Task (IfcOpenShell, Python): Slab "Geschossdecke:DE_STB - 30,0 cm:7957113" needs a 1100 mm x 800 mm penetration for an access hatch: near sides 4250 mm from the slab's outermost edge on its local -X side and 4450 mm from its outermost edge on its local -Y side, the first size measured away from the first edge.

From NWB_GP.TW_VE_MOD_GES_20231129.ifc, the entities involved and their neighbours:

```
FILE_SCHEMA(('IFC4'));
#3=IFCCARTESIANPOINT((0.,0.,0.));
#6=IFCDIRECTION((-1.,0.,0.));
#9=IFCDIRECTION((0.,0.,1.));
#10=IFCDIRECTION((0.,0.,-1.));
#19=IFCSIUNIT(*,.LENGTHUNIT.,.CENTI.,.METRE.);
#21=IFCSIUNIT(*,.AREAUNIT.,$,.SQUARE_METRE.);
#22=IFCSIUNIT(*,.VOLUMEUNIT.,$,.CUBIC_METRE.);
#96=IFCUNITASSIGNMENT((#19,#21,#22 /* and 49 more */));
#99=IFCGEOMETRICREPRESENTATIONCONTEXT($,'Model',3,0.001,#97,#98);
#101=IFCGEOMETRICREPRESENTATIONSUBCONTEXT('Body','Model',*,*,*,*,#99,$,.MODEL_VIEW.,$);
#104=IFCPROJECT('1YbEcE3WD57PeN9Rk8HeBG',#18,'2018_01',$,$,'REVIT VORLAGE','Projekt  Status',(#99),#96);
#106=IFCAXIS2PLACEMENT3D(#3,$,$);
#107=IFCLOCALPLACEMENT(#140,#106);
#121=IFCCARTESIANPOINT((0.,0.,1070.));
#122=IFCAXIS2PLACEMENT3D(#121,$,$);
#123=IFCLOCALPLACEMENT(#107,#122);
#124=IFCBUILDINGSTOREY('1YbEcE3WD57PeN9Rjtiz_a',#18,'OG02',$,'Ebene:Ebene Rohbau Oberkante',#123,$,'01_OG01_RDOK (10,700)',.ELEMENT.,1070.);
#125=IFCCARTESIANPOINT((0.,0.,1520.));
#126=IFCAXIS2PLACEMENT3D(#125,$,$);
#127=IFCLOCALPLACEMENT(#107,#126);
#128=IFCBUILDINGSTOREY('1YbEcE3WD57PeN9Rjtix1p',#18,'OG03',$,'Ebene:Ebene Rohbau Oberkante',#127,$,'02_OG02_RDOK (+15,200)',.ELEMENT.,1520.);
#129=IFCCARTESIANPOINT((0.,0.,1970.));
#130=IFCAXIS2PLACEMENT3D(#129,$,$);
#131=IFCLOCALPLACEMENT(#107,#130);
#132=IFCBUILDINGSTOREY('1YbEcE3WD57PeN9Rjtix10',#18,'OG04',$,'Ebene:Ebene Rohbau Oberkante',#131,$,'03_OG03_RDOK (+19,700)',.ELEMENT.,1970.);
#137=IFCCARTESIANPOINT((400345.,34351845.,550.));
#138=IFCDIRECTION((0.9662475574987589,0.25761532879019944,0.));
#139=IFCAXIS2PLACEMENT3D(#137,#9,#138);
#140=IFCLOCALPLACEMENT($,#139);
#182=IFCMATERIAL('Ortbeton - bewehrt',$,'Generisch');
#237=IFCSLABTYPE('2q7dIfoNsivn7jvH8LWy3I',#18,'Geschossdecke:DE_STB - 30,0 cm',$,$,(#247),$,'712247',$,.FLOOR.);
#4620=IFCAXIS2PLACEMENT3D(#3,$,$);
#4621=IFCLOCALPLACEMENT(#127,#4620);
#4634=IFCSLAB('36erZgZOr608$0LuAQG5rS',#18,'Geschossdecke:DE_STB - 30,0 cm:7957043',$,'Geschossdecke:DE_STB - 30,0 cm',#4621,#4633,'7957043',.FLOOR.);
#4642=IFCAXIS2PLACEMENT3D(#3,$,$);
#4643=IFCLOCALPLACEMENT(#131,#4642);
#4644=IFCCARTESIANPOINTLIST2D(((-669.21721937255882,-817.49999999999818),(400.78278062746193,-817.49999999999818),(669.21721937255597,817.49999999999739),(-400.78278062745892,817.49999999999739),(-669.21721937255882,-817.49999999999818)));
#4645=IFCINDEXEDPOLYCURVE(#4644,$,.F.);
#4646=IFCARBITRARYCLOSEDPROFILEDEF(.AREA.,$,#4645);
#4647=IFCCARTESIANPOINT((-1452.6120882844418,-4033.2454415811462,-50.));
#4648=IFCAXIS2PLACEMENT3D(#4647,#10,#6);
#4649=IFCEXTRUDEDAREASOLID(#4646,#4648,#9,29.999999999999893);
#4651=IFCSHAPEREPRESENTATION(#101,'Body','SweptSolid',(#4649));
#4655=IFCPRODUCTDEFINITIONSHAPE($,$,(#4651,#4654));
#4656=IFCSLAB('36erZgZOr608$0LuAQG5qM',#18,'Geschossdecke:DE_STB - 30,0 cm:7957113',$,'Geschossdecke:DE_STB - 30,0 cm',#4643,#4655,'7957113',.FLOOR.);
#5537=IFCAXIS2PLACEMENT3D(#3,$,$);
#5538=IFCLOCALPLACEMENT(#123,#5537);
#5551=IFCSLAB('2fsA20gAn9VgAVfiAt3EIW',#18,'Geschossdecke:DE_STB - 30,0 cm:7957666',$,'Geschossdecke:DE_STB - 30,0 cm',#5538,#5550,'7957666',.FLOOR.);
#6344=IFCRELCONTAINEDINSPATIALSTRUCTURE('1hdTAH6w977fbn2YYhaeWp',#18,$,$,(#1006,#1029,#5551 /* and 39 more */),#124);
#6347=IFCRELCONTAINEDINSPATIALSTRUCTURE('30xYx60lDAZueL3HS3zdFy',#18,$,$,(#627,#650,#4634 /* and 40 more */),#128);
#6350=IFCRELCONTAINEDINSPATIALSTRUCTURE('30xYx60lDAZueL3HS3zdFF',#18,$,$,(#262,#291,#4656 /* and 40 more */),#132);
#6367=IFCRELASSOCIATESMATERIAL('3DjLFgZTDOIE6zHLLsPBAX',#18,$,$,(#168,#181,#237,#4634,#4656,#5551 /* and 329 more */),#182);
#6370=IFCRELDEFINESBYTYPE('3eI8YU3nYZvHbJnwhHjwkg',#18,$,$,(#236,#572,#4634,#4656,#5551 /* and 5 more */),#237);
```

```python
import numpy as np
import ifcopenshell
import ifcopenshell.api.feature
import ifcopenshell.api.geometry
import ifcopenshell.api.root
import ifcopenshell.geom
import ifcopenshell.util.placement
import ifcopenshell.util.representation
import ifcopenshell.util.shape
import ifcopenshell.util.unit

model = ifcopenshell.open("NWB_GP.TW_VE_MOD_GES_20231129.ifc")
unit_scale = ifcopenshell.util.unit.calculate_unit_scale(model)
settings = ifcopenshell.geom.settings()


def volume(element):
    """Net volume in cubic metres, openings subtracted."""
    shape = ifcopenshell.geom.create_shape(settings, element)
    return ifcopenshell.util.shape.get_volume(shape.geometry)


slab = model.by_id(4656)
before = volume(slab)

# Extent in the slab's own axes, in metres. The edges named are its -X and -Y sides.
slab_shape = ifcopenshell.geom.create_shape(settings, slab)
vertices = ifcopenshell.util.shape.get_vertices(slab_shape.geometry)
x_min, y_min, bottom = vertices.min(axis=0)
top = vertices[:, 2].max()

opening = ifcopenshell.api.root.create_entity(model, ifc_class="IfcOpeningElement", name="Access hatch opening", predefined_type="OPENING")
context = ifcopenshell.util.representation.get_context(model, "Model", "Body", "MODEL_VIEW")
width, depth = 1.1, 0.8
outline = [(0.0, 0.0), (width, 0.0), (width, depth), (0.0, depth), (0.0, 0.0)]
# Overshoot both faces by 50 mm so the cut is clean.
shape = ifcopenshell.api.geometry.add_slab_representation(
    model, context=context, depth=top - bottom + 0.1, polyline=outline
)
ifcopenshell.api.geometry.assign_representation(model, product=opening, representation=shape)

matrix = ifcopenshell.util.placement.get_local_placement(slab.ObjectPlacement)
matrix[:, 3] = matrix @ np.append(np.array([x_min + 4.25, y_min + 4.45, bottom - 0.05]) / unit_scale, 1.0)
ifcopenshell.api.geometry.edit_object_placement(model, product=opening, matrix=matrix, is_si=False)
ifcopenshell.api.feature.add_feature(model, feature=opening, element=slab)

after = volume(slab)

print(f"slab volume {before:.3f} -> {after:.3f} m3")

model.write("NWB_GP.TW_VE_MOD_GES_20231129_rev.ifc")
```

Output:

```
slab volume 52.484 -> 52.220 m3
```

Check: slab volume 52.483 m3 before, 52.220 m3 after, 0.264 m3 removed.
